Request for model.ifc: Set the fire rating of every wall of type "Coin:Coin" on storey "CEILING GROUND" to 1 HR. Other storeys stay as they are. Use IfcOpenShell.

First a look at what the model holds.

```python
import ifcopenshell
import ifcopenshell.util.element

model = ifcopenshell.open("model.ifc")
print(model.schema)
storey = next(s for s in model.by_type("IfcBuildingStorey") if s.Name == "CEILING GROUND")
walls = [e for e in ifcopenshell.util.element.get_decomposition(storey) if e.is_a("IfcWall")]
seen = {}
for e in walls:
    element_type = ifcopenshell.util.element.get_type(e)
    key = (element_type.Name if element_type != e and element_type else None, ifcopenshell.util.element.get_pset(e, "Pset_WallCommon", "FireRating"))
    seen[key] = seen.get(key, 0) + 1
for (name, value), count in sorted(seen.items(), key=str):
    print(count, "x", name, "|", value)
```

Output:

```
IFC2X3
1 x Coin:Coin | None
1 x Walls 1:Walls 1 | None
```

```python
import ifcopenshell
import ifcopenshell.api.pset
import ifcopenshell.util.element

model = ifcopenshell.open("model.ifc")

storey = next(s for s in model.by_type("IfcBuildingStorey") if s.Name == "CEILING GROUND")
walls = [e for e in ifcopenshell.util.element.get_decomposition(storey) if e.is_a("IfcWall")]

count = 0
for e in walls:
    element_type = ifcopenshell.util.element.get_type(e)
    if element_type in (None, e) or element_type.Name != "Coin:Coin":
        continue
    # add_pset returns the element's existing set when there is one.
    pset = ifcopenshell.api.pset.add_pset(model, product=e, name="Pset_WallCommon")
    ifcopenshell.api.pset.edit_pset(model, pset=pset, properties={"FireRating": "1 HR"})
    count += 1

print(count, "walls updated")

model.write("model_edited.ifc")
```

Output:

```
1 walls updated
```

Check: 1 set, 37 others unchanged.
